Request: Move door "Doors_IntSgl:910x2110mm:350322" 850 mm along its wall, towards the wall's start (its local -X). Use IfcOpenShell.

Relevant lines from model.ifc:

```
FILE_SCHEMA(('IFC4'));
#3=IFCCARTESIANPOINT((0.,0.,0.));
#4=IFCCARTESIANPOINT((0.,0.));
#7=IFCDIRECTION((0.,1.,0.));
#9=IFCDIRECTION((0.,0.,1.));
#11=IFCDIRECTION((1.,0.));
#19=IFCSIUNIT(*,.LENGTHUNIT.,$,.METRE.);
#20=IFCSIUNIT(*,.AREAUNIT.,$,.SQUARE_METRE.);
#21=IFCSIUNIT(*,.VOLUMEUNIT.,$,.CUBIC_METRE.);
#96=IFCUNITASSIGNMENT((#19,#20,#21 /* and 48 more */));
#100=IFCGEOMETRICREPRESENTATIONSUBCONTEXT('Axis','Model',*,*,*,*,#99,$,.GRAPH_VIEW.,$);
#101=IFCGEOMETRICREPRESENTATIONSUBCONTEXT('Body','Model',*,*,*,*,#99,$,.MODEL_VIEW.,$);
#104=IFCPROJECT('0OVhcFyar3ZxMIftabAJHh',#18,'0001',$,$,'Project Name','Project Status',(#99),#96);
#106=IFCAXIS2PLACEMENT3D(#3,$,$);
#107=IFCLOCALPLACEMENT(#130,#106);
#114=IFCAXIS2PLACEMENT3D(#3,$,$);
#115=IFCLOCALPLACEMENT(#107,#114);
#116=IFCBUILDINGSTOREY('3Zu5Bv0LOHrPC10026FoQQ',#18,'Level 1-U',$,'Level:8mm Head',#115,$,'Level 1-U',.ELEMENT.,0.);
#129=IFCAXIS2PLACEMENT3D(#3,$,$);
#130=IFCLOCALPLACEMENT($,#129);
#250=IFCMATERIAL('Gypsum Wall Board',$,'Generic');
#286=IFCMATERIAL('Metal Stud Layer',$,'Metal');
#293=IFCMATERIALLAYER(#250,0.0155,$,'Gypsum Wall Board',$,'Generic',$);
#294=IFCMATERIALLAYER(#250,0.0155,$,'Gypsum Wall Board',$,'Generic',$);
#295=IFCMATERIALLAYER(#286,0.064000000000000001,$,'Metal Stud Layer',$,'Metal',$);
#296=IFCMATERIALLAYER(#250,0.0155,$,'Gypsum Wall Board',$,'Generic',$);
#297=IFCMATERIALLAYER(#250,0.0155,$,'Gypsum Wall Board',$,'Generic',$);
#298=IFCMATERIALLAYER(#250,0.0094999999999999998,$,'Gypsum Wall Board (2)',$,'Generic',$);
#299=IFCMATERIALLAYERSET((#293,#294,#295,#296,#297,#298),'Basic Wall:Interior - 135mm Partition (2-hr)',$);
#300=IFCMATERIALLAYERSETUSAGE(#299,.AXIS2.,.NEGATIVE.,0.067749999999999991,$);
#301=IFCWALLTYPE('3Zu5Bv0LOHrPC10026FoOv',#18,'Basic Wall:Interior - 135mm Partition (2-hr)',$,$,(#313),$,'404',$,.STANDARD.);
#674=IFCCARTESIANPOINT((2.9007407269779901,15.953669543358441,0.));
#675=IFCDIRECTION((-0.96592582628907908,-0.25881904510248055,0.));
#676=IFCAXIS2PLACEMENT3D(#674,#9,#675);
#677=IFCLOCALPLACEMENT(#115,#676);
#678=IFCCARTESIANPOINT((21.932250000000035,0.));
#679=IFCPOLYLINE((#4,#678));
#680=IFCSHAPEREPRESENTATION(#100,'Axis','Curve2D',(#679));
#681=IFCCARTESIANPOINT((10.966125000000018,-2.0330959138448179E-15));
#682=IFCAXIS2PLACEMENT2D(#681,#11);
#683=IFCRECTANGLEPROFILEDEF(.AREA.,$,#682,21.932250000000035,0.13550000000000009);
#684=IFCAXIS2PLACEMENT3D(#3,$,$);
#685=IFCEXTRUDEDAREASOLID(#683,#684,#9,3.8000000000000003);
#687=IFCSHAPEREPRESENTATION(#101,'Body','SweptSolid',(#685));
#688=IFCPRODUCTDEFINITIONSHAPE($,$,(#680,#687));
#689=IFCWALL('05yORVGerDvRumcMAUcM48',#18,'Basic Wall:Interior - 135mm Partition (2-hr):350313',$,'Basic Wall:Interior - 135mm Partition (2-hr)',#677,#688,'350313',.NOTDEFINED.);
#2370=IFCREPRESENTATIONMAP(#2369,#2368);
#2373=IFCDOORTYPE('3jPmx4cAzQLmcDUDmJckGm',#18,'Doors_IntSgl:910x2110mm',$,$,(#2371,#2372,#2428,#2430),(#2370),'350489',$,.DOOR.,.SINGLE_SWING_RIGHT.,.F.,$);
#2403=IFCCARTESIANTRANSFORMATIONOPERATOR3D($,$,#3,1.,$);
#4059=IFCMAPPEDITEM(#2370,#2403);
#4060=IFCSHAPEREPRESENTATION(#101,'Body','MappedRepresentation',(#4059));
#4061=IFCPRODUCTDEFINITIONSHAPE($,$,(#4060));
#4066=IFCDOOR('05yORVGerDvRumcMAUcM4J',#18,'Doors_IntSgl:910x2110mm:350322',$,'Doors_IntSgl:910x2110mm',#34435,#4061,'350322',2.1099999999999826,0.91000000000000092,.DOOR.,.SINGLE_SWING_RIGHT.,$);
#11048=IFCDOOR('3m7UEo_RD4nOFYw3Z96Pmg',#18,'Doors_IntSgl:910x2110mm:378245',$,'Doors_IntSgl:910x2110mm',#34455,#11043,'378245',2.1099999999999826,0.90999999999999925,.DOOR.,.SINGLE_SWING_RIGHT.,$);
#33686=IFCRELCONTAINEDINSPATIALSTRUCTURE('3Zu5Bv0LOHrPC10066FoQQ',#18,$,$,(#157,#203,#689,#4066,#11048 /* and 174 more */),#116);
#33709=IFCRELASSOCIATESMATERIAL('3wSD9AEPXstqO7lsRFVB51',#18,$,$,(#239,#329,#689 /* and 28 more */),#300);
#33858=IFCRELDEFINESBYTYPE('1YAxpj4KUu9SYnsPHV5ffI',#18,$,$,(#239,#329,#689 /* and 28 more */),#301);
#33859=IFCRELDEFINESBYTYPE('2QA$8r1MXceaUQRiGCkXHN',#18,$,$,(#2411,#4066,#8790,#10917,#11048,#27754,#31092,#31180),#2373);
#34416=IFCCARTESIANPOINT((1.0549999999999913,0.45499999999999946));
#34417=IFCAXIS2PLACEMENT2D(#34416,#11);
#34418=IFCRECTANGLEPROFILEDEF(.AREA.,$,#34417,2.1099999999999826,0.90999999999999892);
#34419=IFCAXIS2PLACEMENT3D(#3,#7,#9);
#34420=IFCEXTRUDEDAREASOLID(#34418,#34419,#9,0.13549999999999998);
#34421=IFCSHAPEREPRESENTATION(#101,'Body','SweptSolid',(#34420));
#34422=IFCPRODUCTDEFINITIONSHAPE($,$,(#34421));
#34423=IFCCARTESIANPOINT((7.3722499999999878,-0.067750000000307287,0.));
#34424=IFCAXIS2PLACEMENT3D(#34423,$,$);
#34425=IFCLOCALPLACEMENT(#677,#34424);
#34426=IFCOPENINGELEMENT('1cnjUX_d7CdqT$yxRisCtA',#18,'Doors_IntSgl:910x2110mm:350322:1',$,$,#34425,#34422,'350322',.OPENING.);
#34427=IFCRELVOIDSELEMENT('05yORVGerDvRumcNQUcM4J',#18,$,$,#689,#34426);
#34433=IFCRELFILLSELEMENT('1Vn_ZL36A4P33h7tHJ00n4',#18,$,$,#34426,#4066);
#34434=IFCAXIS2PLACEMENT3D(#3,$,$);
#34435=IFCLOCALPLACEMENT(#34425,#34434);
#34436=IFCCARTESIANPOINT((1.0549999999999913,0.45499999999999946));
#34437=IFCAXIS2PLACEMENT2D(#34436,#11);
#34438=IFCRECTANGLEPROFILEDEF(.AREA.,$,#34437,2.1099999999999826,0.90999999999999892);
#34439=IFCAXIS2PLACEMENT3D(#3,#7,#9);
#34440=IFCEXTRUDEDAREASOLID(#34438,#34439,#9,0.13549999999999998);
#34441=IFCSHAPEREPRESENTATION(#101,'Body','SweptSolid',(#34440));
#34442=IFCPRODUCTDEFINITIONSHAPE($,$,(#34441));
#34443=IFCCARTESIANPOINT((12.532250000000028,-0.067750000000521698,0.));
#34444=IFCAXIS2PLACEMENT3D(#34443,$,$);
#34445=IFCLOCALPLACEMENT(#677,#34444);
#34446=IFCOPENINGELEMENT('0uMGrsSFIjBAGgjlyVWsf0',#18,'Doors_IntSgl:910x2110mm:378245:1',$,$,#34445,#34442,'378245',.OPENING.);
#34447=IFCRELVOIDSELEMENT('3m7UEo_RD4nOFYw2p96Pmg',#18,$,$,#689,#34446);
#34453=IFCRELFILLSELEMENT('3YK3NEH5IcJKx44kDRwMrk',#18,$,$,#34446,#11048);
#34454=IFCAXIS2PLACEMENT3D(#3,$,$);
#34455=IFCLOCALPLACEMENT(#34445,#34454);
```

```python
import ifcopenshell
import ifcopenshell.api.geometry
import ifcopenshell.util.placement

model = ifcopenshell.open("model.ifc")

door = model.by_id(4066)
opening = door.FillsVoids[0].RelatingOpeningElement
wall = opening.VoidsElements[0].RelatingBuildingElement

wall_matrix = ifcopenshell.util.placement.get_local_placement(wall.ObjectPlacement)
shift = wall_matrix[:3, 0] * -0.85
before = ifcopenshell.util.placement.get_local_placement(door.ObjectPlacement)[:3, 3].copy()

# The door is placed relative to its opening, so it follows when the opening moves.
matrix = ifcopenshell.util.placement.get_local_placement(opening.ObjectPlacement)
matrix[:3, 3] += shift
ifcopenshell.api.geometry.edit_object_placement(
    model, product=opening, matrix=matrix, is_si=False, should_transform_children=True
)

after = ifcopenshell.util.placement.get_local_placement(door.ObjectPlacement)[:3, 3]
print("door moved by", (after - before).round(3) + 0.0)

model.write("model_edited.ifc")
```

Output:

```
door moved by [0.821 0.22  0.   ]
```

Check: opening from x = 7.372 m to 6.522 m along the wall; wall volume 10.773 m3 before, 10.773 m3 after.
